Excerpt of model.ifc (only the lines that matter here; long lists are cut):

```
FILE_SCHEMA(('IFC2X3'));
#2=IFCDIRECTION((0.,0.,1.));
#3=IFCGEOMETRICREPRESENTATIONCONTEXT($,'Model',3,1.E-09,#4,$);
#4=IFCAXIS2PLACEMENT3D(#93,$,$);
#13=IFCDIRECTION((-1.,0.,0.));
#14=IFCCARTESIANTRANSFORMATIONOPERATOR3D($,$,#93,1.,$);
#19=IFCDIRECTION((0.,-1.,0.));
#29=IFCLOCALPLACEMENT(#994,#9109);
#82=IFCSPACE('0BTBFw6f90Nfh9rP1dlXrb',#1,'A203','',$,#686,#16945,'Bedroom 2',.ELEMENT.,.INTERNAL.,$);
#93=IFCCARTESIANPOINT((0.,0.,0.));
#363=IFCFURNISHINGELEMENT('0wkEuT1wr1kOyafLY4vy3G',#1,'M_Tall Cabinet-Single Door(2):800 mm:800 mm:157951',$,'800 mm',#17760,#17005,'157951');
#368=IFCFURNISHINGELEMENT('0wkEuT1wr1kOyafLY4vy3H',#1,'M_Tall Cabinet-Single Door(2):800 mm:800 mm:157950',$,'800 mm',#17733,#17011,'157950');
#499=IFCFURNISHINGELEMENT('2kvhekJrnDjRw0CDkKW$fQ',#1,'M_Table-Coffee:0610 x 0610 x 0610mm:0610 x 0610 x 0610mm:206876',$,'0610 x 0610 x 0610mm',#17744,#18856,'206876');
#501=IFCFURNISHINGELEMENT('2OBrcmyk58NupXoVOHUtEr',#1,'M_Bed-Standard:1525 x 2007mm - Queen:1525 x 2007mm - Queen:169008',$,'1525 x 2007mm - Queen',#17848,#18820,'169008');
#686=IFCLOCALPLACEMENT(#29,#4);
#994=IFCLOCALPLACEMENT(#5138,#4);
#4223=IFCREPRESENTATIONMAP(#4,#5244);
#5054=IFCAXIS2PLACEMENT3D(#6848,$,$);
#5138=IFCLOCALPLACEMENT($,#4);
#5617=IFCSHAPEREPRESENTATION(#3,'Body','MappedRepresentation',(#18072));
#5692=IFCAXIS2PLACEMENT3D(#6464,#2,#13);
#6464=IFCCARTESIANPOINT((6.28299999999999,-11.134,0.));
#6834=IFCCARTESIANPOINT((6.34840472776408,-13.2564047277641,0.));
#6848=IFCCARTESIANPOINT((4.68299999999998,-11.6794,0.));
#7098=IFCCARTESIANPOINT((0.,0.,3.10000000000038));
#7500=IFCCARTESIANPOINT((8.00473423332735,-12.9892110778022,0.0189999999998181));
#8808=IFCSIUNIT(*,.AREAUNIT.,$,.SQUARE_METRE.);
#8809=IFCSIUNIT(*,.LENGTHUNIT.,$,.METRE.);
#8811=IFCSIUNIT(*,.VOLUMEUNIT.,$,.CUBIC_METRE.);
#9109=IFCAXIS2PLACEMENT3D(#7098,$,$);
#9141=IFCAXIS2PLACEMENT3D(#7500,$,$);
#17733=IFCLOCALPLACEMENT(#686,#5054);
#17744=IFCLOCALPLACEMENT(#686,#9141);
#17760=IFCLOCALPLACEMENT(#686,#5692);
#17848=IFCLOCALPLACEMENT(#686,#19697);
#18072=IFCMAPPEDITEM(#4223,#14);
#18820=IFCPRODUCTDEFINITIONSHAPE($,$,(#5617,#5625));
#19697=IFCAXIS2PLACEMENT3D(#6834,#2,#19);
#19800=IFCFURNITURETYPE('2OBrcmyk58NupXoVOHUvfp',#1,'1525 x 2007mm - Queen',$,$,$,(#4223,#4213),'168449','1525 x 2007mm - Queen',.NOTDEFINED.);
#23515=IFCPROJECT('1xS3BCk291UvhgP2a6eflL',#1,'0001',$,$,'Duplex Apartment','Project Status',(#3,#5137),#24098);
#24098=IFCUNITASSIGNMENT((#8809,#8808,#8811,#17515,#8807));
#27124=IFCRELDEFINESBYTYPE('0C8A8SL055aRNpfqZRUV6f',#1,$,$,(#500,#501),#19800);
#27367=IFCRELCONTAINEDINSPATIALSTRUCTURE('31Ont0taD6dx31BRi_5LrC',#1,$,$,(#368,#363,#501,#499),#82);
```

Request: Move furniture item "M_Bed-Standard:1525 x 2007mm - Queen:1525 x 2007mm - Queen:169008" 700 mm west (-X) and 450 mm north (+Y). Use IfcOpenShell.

```python
import ifcopenshell
import ifcopenshell.api.geometry
import ifcopenshell.util.placement
import ifcopenshell.util.unit

model = ifcopenshell.open("model.ifc")
unit_scale = ifcopenshell.util.unit.calculate_unit_scale(model)

item = model.by_id(501)
matrix = ifcopenshell.util.placement.get_local_placement(item.ObjectPlacement)
matrix[0, 3] -= 0.7 / unit_scale
matrix[1, 3] += 0.45 / unit_scale
ifcopenshell.api.geometry.edit_object_placement(model, product=item, matrix=matrix, is_si=False)

print(ifcopenshell.util.placement.get_local_placement(item.ObjectPlacement).round(3) + 0.0)

model.write("model_v2.ifc")
```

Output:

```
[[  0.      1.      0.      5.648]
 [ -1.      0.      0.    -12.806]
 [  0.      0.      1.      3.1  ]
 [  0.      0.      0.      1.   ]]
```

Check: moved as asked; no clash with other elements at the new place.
